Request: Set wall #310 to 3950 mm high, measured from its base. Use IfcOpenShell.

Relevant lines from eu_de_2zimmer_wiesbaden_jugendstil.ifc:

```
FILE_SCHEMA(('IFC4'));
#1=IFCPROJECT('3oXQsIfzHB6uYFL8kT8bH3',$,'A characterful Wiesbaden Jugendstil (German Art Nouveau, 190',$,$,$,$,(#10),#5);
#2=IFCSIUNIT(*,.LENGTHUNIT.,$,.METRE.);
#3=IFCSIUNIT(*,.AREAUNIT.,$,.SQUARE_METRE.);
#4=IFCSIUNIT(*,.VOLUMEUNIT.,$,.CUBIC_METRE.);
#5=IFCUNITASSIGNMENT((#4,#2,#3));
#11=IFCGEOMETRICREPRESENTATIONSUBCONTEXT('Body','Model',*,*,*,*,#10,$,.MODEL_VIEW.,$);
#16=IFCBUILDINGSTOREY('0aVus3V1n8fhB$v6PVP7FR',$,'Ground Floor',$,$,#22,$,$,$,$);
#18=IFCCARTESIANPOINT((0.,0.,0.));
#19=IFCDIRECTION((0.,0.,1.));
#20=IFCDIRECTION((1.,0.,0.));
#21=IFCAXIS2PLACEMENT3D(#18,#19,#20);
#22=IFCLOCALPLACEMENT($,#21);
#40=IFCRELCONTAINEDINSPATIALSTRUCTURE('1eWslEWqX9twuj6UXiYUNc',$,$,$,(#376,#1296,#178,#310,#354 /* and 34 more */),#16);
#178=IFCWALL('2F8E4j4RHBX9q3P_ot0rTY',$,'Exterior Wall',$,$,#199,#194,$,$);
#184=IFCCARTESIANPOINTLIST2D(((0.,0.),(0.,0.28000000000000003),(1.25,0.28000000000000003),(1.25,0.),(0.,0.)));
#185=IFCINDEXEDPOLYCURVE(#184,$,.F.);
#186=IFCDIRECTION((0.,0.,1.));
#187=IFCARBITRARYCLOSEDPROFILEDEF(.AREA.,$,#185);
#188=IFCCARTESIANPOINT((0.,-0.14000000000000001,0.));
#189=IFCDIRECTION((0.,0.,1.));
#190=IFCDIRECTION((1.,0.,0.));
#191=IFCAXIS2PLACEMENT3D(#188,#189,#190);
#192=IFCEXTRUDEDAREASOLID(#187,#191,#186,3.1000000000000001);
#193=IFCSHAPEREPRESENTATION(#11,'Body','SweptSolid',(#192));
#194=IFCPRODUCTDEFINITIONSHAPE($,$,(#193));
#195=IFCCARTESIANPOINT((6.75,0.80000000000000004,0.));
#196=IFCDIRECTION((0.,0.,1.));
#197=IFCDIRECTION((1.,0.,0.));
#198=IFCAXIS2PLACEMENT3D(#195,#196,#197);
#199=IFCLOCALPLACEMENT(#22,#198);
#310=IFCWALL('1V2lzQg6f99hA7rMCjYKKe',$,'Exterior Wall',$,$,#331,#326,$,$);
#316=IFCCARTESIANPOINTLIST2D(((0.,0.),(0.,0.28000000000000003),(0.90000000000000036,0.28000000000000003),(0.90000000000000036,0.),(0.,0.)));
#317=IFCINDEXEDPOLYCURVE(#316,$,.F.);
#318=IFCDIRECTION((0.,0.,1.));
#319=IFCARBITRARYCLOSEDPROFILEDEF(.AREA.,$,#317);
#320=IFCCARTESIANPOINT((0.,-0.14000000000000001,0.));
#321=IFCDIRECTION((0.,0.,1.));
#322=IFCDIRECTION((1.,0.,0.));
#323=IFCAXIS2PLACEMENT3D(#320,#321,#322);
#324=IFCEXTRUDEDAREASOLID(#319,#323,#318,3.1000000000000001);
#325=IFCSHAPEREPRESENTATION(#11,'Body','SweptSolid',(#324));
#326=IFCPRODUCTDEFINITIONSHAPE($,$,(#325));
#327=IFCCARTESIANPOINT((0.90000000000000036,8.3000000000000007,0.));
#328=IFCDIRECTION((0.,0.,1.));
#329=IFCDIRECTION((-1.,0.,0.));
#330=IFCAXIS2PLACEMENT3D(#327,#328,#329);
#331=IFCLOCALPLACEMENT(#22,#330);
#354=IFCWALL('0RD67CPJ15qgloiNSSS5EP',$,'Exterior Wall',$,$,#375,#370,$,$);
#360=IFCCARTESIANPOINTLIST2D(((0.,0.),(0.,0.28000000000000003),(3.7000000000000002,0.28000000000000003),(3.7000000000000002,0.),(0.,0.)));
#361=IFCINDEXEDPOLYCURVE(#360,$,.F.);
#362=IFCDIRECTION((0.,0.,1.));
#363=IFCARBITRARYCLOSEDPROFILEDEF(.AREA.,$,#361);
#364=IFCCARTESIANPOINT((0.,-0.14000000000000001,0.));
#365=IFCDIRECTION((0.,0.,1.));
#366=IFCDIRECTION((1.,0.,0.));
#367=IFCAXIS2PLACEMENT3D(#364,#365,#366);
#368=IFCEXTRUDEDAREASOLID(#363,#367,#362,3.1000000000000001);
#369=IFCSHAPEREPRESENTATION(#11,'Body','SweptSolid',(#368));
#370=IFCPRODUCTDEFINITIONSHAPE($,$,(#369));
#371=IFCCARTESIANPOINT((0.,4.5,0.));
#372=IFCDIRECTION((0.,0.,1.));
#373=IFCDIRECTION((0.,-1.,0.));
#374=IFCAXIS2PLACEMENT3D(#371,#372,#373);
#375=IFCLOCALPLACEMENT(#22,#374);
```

```python
import ifcopenshell
import ifcopenshell.geom
import ifcopenshell.util.representation
import ifcopenshell.util.shape

model = ifcopenshell.open("eu_de_2zimmer_wiesbaden_jugendstil.ifc")
settings = ifcopenshell.geom.settings()


def volume(element):
    """Net volume in cubic metres, openings subtracted."""
    shape = ifcopenshell.geom.create_shape(settings, element)
    return ifcopenshell.util.shape.get_volume(shape.geometry)


wall = model.by_guid("1V2lzQg6f99hA7rMCjYKKe")
before = volume(wall)

body = ifcopenshell.util.representation.get_representation(wall, "Model", "Body")
solid = body.Items[0]
old_height = solid.Depth
solid.Depth = 3.95
after = volume(wall)

print(f"height {old_height:g} -> {solid.Depth:g}, volume {before:.3f} -> {after:.3f} m3")

model.write("eu_de_2zimmer_wiesbaden_jugendstil_rev.ifc")
```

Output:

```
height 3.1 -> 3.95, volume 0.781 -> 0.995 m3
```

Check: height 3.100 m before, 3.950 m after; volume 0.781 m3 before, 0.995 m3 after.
